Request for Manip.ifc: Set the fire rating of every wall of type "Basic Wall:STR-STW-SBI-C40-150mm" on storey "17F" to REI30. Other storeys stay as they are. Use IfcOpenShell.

First a look at what the model holds.

```python
import ifcopenshell
import ifcopenshell.util.element

model = ifcopenshell.open("Manip.ifc")
print(model.schema)
storey = next(s for s in model.by_type("IfcBuildingStorey") if s.Name == "17F")
walls = [e for e in ifcopenshell.util.element.get_decomposition(storey) if e.is_a("IfcWall")]
seen = {}
for e in walls:
    element_type = ifcopenshell.util.element.get_type(e)
    key = (element_type.Name if element_type != e and element_type else None, ifcopenshell.util.element.get_pset(e, "Pset_WallCommon", "FireRating"))
    seen[key] = seen.get(key, 0) + 1
for (name, value), count in sorted(seen.items(), key=str):
    print(count, "x", name, "|", value)
```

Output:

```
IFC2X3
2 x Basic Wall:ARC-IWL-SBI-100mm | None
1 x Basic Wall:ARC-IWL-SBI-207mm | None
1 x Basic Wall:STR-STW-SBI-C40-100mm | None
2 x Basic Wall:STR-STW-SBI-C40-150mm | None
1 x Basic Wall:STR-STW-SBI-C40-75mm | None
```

```python
import ifcopenshell
import ifcopenshell.api.pset
import ifcopenshell.util.element

model = ifcopenshell.open("Manip.ifc")

storey = next(s for s in model.by_type("IfcBuildingStorey") if s.Name == "17F")
walls = [e for e in ifcopenshell.util.element.get_decomposition(storey) if e.is_a("IfcWall")]

count = 0
for e in walls:
    element_type = ifcopenshell.util.element.get_type(e)
    if element_type in (None, e) or element_type.Name != "Basic Wall:STR-STW-SBI-C40-150mm":
        continue
    # add_pset returns the element's existing set when there is one.
    pset = ifcopenshell.api.pset.add_pset(model, product=e, name="Pset_WallCommon")
    ifcopenshell.api.pset.edit_pset(model, pset=pset, properties={"FireRating": "REI30"})
    count += 1

print(count, "walls updated")

model.write("Manip_edited.ifc")
```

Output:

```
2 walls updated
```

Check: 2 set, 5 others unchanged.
